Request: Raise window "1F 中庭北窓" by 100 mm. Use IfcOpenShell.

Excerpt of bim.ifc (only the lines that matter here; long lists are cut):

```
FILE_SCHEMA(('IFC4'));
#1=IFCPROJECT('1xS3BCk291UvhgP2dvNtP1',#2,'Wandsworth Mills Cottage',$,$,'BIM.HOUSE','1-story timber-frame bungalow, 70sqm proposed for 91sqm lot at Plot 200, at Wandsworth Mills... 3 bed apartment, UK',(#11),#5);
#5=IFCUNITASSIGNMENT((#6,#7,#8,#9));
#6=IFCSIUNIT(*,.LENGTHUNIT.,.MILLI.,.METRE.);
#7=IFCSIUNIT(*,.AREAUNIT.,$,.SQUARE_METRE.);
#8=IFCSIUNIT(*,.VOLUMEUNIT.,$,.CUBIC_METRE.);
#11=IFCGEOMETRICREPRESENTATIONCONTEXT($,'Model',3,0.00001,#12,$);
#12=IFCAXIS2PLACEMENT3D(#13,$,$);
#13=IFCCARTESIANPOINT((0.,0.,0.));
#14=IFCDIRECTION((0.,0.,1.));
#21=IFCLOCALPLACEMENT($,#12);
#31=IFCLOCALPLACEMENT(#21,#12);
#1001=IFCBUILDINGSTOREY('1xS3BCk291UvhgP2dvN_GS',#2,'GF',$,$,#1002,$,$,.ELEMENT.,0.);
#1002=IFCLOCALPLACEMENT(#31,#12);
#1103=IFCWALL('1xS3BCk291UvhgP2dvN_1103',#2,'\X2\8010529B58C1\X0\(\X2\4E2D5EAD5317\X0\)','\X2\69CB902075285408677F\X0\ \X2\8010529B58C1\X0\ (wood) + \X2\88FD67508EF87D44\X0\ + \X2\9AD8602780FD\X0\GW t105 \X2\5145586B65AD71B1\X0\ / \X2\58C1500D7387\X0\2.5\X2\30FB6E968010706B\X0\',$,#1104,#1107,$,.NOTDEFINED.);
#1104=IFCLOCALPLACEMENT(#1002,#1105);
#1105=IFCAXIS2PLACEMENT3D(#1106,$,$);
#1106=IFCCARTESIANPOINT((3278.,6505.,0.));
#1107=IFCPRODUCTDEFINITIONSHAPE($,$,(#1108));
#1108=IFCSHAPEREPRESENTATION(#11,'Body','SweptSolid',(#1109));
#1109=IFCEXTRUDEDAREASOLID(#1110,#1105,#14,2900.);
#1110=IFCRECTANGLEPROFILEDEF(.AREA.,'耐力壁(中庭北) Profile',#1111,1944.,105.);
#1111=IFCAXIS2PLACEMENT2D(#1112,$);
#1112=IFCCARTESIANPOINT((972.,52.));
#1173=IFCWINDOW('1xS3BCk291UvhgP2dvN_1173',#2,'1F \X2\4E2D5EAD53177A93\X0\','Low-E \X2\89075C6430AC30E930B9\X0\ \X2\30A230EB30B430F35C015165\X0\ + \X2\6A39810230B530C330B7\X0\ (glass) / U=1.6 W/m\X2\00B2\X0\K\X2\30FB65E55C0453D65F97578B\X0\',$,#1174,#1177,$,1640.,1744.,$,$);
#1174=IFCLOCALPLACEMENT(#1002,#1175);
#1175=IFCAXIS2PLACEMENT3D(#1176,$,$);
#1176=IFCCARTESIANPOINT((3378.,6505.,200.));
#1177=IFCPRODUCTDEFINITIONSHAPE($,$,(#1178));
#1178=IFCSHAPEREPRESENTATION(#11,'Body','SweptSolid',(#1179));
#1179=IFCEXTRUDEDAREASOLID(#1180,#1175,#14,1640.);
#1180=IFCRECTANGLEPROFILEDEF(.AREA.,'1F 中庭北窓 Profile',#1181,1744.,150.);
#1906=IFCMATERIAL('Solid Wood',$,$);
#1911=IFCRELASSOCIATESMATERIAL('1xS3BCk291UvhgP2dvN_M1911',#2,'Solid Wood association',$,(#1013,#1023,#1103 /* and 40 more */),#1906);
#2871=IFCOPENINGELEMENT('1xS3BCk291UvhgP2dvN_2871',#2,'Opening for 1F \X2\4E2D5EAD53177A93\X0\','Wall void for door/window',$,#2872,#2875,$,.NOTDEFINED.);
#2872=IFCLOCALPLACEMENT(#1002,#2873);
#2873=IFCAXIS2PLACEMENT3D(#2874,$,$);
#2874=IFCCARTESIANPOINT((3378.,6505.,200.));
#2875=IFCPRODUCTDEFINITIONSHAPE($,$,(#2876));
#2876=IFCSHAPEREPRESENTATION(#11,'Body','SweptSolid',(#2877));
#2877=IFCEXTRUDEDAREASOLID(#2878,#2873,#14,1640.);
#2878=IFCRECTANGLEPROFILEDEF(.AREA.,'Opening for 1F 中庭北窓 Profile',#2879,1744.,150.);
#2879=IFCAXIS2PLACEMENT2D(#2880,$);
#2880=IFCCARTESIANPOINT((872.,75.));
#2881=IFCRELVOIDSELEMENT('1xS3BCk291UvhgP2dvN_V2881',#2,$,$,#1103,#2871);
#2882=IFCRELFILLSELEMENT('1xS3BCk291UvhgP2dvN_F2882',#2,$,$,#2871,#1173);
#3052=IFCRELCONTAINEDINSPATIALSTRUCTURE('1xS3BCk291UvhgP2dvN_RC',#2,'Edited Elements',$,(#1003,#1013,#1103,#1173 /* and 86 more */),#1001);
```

```python
import numpy as np
import ifcopenshell
import ifcopenshell.api.geometry
import ifcopenshell.util.placement
import ifcopenshell.util.unit

model = ifcopenshell.open("bim.ifc")
unit_scale = ifcopenshell.util.unit.calculate_unit_scale(model)

window = model.by_guid("1xS3BCk291UvhgP2dvN_1173")
opening = window.FillsVoids[0].RelatingOpeningElement
dz = 0.1 / unit_scale

shift = np.array([0.0, 0.0, dz])
# The window is not placed relative to its opening, so move both.
for product in (opening, window):
    matrix = ifcopenshell.util.placement.get_local_placement(product.ObjectPlacement)
    matrix[:3, 3] += shift
    ifcopenshell.api.geometry.edit_object_placement(model, product=product, matrix=matrix, is_si=False)

print(f"moved by {dz * unit_scale:+.3f} m")

model.write("bim-out.ifc")
```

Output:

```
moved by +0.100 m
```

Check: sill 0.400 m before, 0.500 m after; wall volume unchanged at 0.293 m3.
